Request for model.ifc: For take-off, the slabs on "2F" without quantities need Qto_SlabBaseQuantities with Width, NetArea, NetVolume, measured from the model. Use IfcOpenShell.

First a look at what the model holds.

```python
import ifcopenshell
import ifcopenshell.util.element
import ifcopenshell.util.unit

model = ifcopenshell.open("model.ifc")
print(model.schema)
for unit_type in ("LENGTHUNIT", "AREAUNIT", "VOLUMEUNIT"):
    print(unit_type, ifcopenshell.util.unit.calculate_unit_scale(model, unit_type))
storey = next(s for s in model.by_type("IfcBuildingStorey") if s.Name == "2F")
slabs = [e for e in ifcopenshell.util.element.get_decomposition(storey) if e.is_a("IfcSlab")]
for e in sorted(slabs, key=lambda e: e.id()):
    print(e.id(), e.is_a(), e.Name, list(ifcopenshell.util.element.get_psets(e, qtos_only=True)), sep=" | ")
```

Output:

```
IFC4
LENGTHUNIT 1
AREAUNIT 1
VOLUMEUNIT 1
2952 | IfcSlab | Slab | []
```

```python
import ifcopenshell
import ifcopenshell.api.pset
import ifcopenshell.geom
import ifcopenshell.util.element
import ifcopenshell.util.shape
import ifcopenshell.util.unit

model = ifcopenshell.open("model.ifc")
unit_scale = ifcopenshell.util.unit.calculate_unit_scale(model)
area_scale = ifcopenshell.util.unit.calculate_unit_scale(model, "AREAUNIT")
volume_scale = ifcopenshell.util.unit.calculate_unit_scale(model, "VOLUMEUNIT")
settings = ifcopenshell.geom.settings()

storey = next(s for s in model.by_type("IfcBuildingStorey") if s.Name == "2F")
slabs = [e for e in ifcopenshell.util.element.get_decomposition(storey) if e.is_a("IfcSlab")]

for e in sorted(slabs, key=lambda e: e.id()):
    if ifcopenshell.util.element.get_psets(e, qtos_only=True, should_inherit=False):
        continue
    # Geometry comes back in metres, in the element's own axes.
    shape = ifcopenshell.geom.create_shape(settings, e)
    values = {
        "Width": ifcopenshell.util.shape.get_z(shape.geometry) / unit_scale,
        "NetArea": ifcopenshell.util.shape.get_footprint_area(shape.geometry) / area_scale,
        "NetVolume": ifcopenshell.util.shape.get_volume(shape.geometry) / volume_scale,
    }
    qto = ifcopenshell.api.pset.add_qto(model, product=e, name="Qto_SlabBaseQuantities")
    ifcopenshell.api.pset.edit_qto(model, qto=qto, properties=values)
    print(e.id(), {k: round(v, 3) for k, v in values.items()})

model.write("model-out.ifc")
```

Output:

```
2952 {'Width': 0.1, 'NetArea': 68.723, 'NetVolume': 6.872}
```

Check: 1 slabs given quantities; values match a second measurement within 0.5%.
